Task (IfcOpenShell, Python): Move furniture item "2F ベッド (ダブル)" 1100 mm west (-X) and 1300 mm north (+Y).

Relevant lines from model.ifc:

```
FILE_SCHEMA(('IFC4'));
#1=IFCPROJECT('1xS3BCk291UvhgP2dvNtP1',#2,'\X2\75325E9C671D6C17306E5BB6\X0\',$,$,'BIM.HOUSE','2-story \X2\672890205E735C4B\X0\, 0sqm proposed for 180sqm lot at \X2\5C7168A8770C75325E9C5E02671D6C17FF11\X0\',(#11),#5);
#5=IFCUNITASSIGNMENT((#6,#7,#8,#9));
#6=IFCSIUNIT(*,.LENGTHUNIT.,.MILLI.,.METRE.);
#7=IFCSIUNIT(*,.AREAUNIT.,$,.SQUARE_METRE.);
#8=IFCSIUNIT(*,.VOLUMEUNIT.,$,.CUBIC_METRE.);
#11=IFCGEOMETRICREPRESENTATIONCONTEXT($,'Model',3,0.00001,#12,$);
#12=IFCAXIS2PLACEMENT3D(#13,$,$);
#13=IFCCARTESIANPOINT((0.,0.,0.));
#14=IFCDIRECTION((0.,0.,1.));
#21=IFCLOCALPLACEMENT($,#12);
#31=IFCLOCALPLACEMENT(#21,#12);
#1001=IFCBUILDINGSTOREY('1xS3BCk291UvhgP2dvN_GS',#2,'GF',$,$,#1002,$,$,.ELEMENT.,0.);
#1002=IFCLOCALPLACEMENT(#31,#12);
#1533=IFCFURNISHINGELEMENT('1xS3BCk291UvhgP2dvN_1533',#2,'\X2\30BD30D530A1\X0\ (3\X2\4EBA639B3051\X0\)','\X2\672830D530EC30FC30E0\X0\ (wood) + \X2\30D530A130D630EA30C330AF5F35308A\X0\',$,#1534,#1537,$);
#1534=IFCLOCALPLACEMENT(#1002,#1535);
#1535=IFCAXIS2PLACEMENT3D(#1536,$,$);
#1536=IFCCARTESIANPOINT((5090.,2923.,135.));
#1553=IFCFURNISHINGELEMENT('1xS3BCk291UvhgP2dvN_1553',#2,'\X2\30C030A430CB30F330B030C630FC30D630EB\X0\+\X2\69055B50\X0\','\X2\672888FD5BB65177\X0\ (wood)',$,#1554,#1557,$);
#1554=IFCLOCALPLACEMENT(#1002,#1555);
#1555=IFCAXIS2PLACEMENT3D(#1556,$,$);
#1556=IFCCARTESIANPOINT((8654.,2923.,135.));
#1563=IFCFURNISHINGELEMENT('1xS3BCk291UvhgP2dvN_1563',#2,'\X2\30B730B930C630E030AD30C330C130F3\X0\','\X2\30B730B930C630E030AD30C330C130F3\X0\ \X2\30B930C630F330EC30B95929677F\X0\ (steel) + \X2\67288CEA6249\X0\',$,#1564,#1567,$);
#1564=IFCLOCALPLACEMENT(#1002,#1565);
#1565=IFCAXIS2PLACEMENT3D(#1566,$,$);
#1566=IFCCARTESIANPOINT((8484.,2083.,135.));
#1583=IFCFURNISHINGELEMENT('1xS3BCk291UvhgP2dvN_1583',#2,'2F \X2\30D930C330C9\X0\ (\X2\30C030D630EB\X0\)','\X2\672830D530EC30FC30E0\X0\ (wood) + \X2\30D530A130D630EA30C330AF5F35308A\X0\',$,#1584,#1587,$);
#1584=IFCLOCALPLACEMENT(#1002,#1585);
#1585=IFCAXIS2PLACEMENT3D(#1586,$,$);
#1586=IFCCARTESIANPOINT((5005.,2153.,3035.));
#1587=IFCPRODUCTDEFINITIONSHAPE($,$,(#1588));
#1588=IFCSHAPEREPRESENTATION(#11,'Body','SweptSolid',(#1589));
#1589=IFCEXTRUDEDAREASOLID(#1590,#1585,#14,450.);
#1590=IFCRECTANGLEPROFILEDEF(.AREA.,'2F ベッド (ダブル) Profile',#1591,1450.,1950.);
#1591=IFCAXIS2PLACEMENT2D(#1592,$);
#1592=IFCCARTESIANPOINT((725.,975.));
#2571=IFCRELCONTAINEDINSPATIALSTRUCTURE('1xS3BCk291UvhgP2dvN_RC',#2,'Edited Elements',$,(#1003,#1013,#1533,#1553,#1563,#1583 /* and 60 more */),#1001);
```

```python
import ifcopenshell
import ifcopenshell.api.geometry
import ifcopenshell.util.placement
import ifcopenshell.util.unit

model = ifcopenshell.open("model.ifc")
unit_scale = ifcopenshell.util.unit.calculate_unit_scale(model)

item = model.by_guid("1xS3BCk291UvhgP2dvN_1583")
matrix = ifcopenshell.util.placement.get_local_placement(item.ObjectPlacement)
matrix[0, 3] -= 1.1 / unit_scale
matrix[1, 3] += 1.3 / unit_scale
ifcopenshell.api.geometry.edit_object_placement(model, product=item, matrix=matrix, is_si=False)

print(ifcopenshell.util.placement.get_local_placement(item.ObjectPlacement).round(3) + 0.0)

model.write("model_rev.ifc")
```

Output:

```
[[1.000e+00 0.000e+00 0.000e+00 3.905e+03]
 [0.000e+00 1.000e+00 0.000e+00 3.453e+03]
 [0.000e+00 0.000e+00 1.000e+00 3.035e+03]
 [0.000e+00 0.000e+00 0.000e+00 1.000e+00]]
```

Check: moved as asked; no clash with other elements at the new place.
